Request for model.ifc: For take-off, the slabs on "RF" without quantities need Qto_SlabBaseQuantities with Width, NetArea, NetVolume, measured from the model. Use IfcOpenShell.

First a look at what the model holds.

```python
import ifcopenshell
import ifcopenshell.util.element
import ifcopenshell.util.unit

model = ifcopenshell.open("model.ifc")
print(model.schema)
for unit_type in ("LENGTHUNIT", "AREAUNIT", "VOLUMEUNIT"):
    print(unit_type, ifcopenshell.util.unit.calculate_unit_scale(model, unit_type))
storey = next(s for s in model.by_type("IfcBuildingStorey") if s.Name == "RF")
slabs = [e for e in ifcopenshell.util.element.get_decomposition(storey) if e.is_a("IfcSlab")]
for e in sorted(slabs, key=lambda e: e.id()):
    print(e.id(), e.is_a(), e.Name, list(ifcopenshell.util.element.get_psets(e, qtos_only=True)), sep=" | ")
```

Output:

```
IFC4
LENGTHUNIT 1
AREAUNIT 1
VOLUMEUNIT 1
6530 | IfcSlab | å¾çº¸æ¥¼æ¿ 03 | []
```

```python
import ifcopenshell
import ifcopenshell.api.pset
import ifcopenshell.geom
import ifcopenshell.util.element
import ifcopenshell.util.shape
import ifcopenshell.util.unit

model = ifcopenshell.open("model.ifc")
unit_scale = ifcopenshell.util.unit.calculate_unit_scale(model)
area_scale = ifcopenshell.util.unit.calculate_unit_scale(model, "AREAUNIT")
volume_scale = ifcopenshell.util.unit.calculate_unit_scale(model, "VOLUMEUNIT")
settings = ifcopenshell.geom.settings()

storey = next(s for s in model.by_type("IfcBuildingStorey") if s.Name == "RF")
slabs = [e for e in ifcopenshell.util.element.get_decomposition(storey) if e.is_a("IfcSlab")]

for e in sorted(slabs, key=lambda e: e.id()):
    if ifcopenshell.util.element.get_psets(e, qtos_only=True, should_inherit=False):
        continue
    # Geometry comes back in metres, in the element's own axes.
    shape = ifcopenshell.geom.create_shape(settings, e)
    values = {
        "Width": ifcopenshell.util.shape.get_z(shape.geometry) / unit_scale,
        "NetArea": ifcopenshell.util.shape.get_footprint_area(shape.geometry) / area_scale,
        "NetVolume": ifcopenshell.util.shape.get_volume(shape.geometry) / volume_scale,
    }
    qto = ifcopenshell.api.pset.add_qto(model, product=e, name="Qto_SlabBaseQuantities")
    ifcopenshell.api.pset.edit_qto(model, qto=qto, properties=values)
    print(e.id(), {k: round(v, 3) for k, v in values.items()})

model.write("model_updated.ifc")
```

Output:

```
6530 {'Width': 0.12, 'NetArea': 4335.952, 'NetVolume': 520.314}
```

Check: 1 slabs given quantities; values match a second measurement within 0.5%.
